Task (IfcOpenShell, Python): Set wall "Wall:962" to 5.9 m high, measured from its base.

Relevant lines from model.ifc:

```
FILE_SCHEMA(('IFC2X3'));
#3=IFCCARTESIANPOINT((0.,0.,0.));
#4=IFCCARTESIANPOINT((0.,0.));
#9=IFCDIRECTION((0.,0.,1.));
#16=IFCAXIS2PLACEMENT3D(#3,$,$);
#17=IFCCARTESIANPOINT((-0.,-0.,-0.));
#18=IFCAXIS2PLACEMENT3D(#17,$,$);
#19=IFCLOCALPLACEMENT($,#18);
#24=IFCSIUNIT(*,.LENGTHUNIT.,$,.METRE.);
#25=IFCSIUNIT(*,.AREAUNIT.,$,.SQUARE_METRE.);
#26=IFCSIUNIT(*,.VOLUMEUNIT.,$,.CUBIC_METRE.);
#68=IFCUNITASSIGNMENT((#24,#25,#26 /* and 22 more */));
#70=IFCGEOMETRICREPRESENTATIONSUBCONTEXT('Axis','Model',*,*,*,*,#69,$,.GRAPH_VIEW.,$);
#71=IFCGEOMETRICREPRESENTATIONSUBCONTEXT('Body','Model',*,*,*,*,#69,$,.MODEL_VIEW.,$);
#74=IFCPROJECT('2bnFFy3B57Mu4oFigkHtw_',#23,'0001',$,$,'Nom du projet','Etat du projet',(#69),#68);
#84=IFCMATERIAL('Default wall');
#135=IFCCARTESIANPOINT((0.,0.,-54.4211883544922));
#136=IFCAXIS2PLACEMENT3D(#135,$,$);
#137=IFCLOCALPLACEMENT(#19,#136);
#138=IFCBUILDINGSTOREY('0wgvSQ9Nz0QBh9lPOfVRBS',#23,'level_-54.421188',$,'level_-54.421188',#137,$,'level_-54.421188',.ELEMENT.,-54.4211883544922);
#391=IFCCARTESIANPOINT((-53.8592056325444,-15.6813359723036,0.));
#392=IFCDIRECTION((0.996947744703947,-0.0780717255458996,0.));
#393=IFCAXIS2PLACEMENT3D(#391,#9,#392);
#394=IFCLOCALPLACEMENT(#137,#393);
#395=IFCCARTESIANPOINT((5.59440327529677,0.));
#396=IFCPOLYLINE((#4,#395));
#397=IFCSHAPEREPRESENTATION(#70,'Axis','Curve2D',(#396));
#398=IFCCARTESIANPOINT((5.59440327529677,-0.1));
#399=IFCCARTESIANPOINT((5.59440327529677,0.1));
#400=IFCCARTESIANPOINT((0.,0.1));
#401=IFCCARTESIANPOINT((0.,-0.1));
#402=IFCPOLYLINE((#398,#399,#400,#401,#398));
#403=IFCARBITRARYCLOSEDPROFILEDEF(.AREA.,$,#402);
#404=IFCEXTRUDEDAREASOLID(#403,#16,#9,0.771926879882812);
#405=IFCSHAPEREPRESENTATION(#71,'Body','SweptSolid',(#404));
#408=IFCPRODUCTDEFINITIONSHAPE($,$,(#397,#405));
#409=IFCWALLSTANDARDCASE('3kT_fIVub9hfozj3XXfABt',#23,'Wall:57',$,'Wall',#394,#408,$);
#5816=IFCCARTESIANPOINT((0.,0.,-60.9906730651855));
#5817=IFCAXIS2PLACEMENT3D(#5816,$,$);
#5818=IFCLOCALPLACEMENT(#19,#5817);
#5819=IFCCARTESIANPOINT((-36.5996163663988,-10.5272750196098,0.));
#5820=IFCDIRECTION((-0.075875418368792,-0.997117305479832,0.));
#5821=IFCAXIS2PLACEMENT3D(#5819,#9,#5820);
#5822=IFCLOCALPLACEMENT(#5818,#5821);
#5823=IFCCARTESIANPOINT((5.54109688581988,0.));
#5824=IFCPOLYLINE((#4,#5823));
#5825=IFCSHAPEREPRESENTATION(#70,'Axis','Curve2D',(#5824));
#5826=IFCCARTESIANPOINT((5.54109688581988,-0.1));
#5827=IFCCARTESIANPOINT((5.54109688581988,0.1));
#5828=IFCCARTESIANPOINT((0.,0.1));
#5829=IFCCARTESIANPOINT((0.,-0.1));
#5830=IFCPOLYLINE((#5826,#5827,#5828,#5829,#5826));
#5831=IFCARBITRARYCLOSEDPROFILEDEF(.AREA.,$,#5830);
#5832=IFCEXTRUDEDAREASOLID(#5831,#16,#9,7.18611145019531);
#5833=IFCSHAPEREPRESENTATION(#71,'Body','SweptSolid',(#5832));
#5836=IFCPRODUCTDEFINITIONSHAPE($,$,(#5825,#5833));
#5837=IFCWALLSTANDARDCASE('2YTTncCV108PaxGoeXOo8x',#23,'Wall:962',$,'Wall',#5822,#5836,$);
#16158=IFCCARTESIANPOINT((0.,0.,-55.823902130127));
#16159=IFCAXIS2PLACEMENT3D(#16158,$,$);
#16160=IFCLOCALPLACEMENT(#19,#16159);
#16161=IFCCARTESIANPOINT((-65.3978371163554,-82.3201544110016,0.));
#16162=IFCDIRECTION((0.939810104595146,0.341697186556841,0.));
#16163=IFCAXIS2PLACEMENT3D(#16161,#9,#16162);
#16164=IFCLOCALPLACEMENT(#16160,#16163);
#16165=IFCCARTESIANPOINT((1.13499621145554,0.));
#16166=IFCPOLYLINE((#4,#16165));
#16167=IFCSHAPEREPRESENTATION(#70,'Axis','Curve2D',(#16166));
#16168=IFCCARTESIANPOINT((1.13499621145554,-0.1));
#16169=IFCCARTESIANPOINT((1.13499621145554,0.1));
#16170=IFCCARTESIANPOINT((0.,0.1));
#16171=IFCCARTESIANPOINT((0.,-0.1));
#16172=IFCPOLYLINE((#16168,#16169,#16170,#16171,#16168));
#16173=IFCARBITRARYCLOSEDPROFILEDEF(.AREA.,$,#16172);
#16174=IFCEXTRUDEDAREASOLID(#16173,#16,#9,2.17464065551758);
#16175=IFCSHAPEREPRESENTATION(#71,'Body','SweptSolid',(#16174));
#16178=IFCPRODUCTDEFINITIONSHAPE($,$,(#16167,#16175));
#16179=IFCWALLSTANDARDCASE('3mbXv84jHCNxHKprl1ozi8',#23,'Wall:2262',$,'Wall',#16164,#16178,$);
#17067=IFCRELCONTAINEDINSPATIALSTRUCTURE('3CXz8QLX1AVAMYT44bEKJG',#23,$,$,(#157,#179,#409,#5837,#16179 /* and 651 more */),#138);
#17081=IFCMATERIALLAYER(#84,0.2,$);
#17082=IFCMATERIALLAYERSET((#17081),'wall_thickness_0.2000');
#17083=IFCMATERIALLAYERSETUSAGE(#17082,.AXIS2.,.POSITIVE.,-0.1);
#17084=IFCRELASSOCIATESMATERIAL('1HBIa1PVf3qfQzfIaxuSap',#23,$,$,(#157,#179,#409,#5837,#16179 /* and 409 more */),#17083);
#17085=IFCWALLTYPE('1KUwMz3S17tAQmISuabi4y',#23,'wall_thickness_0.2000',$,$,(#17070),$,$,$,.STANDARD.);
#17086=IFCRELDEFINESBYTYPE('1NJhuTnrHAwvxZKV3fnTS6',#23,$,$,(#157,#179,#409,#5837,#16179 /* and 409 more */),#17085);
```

```python
import ifcopenshell
import ifcopenshell.geom
import ifcopenshell.util.representation
import ifcopenshell.util.shape

model = ifcopenshell.open("model.ifc")
settings = ifcopenshell.geom.settings()


def volume(element):
    """Net volume in cubic metres, openings subtracted."""
    shape = ifcopenshell.geom.create_shape(settings, element)
    return ifcopenshell.util.shape.get_volume(shape.geometry)


wall = model.by_id(5837)
before = volume(wall)

body = ifcopenshell.util.representation.get_representation(wall, "Model", "Body")
solid = body.Items[0]
old_height = solid.Depth
solid.Depth = 5.9
after = volume(wall)

print(f"height {old_height:g} -> {solid.Depth:g}, volume {before:.3f} -> {after:.3f} m3")

model.write("model_rev.ifc")
```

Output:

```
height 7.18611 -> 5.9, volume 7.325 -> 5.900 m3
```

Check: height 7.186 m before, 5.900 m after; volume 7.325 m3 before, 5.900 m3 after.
